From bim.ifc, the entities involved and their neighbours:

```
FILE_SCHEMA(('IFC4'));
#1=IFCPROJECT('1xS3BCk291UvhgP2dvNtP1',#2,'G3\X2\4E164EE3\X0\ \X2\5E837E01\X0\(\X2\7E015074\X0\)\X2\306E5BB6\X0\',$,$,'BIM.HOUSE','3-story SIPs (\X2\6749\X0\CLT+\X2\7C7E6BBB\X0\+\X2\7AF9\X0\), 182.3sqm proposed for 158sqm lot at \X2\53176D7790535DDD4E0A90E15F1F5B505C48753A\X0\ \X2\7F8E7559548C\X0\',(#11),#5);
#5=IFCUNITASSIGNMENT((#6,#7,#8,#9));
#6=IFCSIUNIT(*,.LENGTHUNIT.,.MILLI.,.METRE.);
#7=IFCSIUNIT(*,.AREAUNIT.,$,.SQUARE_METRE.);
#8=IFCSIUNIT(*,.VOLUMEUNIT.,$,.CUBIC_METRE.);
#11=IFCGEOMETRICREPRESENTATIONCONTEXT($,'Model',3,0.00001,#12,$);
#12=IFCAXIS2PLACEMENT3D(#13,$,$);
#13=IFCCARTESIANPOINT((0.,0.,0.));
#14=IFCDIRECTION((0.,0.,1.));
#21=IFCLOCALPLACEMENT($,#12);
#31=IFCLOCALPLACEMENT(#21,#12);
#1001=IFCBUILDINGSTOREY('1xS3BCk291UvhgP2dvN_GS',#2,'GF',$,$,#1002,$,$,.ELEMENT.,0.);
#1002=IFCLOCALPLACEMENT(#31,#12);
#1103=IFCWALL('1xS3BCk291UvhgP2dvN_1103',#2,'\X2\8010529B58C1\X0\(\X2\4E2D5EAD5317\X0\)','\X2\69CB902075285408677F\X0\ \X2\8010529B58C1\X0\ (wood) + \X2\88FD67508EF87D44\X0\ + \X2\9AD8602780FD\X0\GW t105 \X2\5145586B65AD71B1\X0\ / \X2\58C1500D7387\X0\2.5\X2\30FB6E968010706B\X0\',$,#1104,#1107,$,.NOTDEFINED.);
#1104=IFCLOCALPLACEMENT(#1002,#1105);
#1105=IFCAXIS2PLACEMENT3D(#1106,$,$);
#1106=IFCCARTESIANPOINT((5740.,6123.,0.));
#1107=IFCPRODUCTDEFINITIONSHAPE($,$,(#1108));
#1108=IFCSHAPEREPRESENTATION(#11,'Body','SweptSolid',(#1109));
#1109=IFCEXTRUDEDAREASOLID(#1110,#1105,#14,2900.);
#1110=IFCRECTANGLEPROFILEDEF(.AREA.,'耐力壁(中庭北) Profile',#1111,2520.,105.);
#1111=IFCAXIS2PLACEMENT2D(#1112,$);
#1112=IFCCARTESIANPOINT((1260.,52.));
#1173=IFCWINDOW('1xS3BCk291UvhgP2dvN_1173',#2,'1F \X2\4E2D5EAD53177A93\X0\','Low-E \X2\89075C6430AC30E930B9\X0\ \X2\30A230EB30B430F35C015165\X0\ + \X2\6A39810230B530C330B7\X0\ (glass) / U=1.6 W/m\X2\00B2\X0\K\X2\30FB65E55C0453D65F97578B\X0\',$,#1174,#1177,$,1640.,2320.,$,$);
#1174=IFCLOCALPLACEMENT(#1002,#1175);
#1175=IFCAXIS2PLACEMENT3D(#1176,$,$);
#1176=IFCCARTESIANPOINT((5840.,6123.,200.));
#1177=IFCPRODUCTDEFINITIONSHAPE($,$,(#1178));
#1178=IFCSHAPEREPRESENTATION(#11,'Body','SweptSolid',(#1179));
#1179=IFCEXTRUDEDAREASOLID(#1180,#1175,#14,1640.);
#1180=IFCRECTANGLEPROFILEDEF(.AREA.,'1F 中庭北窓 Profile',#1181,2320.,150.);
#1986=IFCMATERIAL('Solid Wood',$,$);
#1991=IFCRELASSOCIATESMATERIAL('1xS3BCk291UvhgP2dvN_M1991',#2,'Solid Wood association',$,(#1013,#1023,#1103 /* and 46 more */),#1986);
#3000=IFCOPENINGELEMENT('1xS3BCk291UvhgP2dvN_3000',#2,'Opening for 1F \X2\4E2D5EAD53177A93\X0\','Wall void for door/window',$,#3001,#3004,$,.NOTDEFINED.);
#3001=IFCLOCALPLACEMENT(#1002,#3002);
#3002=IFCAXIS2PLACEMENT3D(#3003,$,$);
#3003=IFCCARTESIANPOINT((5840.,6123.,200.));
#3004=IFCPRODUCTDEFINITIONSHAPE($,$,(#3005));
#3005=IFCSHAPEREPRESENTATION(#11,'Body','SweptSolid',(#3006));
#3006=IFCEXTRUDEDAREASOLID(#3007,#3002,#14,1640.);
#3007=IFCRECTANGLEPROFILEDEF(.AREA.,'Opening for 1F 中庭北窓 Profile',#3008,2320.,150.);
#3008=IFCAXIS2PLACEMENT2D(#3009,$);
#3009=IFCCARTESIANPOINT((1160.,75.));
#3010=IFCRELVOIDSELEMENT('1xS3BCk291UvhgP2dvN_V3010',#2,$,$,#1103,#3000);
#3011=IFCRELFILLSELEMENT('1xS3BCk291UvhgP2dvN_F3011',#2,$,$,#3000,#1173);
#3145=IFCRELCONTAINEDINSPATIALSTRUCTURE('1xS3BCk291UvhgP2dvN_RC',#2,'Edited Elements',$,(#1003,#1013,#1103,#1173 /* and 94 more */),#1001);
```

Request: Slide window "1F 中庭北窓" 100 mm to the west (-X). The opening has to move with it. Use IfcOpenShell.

```python
import ifcopenshell
import ifcopenshell.api.geometry
import ifcopenshell.util.placement

model = ifcopenshell.open("bim.ifc")

window = model.by_guid("1xS3BCk291UvhgP2dvN_1173")
opening = window.FillsVoids[0].RelatingOpeningElement
wall = opening.VoidsElements[0].RelatingBuildingElement

wall_matrix = ifcopenshell.util.placement.get_local_placement(wall.ObjectPlacement)
shift = wall_matrix[:3, 0] * -100.0
before = ifcopenshell.util.placement.get_local_placement(window.ObjectPlacement)[:3, 3].copy()

# The window is not placed relative to its opening, so move both.
for product in (opening, window):
    matrix = ifcopenshell.util.placement.get_local_placement(product.ObjectPlacement)
    matrix[:3, 3] += shift
    ifcopenshell.api.geometry.edit_object_placement(model, product=product, matrix=matrix, is_si=False)

after = ifcopenshell.util.placement.get_local_placement(window.ObjectPlacement)[:3, 3]
print("window moved by", (after - before).round(3) + 0.0)

model.write("bim-out.ifc")
```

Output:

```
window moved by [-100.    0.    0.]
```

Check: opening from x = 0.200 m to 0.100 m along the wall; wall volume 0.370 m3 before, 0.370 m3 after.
